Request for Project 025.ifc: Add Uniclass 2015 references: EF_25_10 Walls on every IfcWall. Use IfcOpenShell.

First a look at what the model holds.

```python
import ifcopenshell

model = ifcopenshell.open("Project 025.ifc")
print(model.schema)
print("classifications:", [c.Name for c in model.by_type("IfcClassification")])
for ifc_class in ("IfcDoor", "IfcRoof", "IfcStair", "IfcWall", "IfcWindow"):
    print(ifc_class, len(model.by_type(ifc_class)))
```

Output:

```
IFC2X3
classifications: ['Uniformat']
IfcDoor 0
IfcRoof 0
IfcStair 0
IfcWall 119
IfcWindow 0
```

```python
import ifcopenshell
import ifcopenshell.api.classification

model = ifcopenshell.open("Project 025.ifc")

# IFC2X3 requires Source and Edition and has no link from the project to the system.
system = model.create_entity("IfcClassification", Source="NBS", Edition="2015", Name="Uniclass 2015")

codes = {
    "IfcWall": ("EF_25_10", "Walls"),
}
for ifc_class, (code, name) in codes.items():
    products = model.by_type(ifc_class)
    ifcopenshell.api.classification.add_reference(
        model, products=products, classification=system, identification=code, name=name
    )
    print(code, len(products))

model.write("Project 025_edited.ifc")
```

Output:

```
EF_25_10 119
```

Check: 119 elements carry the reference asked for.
